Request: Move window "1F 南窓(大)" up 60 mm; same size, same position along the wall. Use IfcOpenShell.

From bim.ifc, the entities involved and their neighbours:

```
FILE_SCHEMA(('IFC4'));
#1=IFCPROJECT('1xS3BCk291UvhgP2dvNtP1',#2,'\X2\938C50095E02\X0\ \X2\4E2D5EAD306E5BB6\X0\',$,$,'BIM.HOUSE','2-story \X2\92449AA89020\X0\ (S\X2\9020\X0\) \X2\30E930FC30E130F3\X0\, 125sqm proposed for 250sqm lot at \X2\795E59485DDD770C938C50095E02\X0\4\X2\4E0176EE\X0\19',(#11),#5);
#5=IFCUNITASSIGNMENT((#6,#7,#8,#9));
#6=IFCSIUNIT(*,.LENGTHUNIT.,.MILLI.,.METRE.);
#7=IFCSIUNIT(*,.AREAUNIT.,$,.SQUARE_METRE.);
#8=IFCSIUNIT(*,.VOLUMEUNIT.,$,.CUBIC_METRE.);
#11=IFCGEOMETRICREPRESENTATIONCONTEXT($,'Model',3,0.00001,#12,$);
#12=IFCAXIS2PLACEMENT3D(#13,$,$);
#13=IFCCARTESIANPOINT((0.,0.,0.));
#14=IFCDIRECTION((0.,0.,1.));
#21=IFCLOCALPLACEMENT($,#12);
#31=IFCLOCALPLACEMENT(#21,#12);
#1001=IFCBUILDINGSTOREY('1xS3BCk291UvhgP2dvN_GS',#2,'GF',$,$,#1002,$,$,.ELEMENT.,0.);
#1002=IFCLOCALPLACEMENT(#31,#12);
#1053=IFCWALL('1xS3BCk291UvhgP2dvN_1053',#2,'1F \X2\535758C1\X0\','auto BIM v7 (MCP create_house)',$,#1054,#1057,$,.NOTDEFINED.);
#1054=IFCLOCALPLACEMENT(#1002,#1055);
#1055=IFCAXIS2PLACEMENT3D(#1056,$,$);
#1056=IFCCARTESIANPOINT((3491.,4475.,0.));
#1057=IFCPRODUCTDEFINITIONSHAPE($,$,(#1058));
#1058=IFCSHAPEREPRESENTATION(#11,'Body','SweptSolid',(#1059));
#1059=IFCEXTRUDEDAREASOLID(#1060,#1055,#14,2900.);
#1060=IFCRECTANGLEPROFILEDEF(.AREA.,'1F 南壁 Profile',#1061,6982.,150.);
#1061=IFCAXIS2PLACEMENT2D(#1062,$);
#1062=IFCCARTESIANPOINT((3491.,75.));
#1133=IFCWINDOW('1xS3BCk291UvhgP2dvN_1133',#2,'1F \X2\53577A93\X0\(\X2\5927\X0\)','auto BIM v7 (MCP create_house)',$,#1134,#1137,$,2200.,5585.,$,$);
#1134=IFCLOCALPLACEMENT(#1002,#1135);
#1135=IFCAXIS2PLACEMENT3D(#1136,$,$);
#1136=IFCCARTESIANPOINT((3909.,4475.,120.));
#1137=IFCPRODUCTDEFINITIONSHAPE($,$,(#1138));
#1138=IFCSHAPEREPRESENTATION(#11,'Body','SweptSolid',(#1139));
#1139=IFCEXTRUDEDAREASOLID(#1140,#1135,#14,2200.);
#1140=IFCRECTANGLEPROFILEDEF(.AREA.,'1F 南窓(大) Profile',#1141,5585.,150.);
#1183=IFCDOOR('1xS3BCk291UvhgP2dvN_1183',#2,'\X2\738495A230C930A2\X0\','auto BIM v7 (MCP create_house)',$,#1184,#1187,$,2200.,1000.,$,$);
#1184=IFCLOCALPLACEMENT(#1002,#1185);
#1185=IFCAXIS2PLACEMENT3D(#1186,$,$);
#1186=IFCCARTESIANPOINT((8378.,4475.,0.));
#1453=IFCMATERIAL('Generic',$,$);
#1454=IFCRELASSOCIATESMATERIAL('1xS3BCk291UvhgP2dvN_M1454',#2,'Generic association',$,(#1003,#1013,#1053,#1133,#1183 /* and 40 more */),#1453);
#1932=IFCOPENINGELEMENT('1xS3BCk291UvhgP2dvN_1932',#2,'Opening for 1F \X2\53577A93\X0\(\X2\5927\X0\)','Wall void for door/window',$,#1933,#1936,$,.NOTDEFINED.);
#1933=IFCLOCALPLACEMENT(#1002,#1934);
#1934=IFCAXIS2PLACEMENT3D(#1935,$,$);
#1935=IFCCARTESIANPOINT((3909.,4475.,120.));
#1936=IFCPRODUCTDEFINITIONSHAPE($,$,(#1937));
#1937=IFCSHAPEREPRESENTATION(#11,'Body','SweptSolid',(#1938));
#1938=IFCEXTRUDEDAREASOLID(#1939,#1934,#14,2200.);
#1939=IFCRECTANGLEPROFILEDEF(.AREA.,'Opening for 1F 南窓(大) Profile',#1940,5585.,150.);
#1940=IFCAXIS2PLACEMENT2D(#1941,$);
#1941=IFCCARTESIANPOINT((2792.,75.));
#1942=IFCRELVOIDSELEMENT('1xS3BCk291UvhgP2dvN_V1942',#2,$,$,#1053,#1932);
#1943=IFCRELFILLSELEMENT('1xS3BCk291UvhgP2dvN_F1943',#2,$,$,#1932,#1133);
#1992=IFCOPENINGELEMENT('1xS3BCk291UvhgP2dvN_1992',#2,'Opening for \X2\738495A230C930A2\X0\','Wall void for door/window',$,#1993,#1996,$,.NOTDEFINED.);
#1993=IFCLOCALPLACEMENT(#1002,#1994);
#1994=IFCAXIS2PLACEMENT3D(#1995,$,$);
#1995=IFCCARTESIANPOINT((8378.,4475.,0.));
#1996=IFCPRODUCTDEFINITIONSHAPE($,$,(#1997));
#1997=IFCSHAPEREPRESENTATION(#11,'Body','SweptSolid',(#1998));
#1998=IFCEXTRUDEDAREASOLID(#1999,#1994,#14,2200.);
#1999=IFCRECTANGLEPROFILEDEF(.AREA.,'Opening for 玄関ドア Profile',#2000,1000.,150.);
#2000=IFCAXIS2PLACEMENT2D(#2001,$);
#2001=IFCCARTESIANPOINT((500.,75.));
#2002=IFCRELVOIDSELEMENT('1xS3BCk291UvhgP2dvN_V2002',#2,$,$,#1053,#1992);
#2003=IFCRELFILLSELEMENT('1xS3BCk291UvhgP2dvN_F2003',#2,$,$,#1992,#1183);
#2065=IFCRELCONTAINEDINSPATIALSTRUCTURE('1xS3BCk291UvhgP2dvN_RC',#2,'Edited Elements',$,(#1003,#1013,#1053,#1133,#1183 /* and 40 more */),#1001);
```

```python
import numpy as np
import ifcopenshell
import ifcopenshell.api.geometry
import ifcopenshell.util.placement
import ifcopenshell.util.unit

model = ifcopenshell.open("bim.ifc")
unit_scale = ifcopenshell.util.unit.calculate_unit_scale(model)

window = model.by_id(1133)
opening = window.FillsVoids[0].RelatingOpeningElement
dz = 0.06 / unit_scale

shift = np.array([0.0, 0.0, dz])
# The window is not placed relative to its opening, so move both.
for product in (opening, window):
    matrix = ifcopenshell.util.placement.get_local_placement(product.ObjectPlacement)
    matrix[:3, 3] += shift
    ifcopenshell.api.geometry.edit_object_placement(model, product=product, matrix=matrix, is_si=False)

print(f"moved by {dz * unit_scale:+.3f} m")

model.write("bim-out.ifc")
```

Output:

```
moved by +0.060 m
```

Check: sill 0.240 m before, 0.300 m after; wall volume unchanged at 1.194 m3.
